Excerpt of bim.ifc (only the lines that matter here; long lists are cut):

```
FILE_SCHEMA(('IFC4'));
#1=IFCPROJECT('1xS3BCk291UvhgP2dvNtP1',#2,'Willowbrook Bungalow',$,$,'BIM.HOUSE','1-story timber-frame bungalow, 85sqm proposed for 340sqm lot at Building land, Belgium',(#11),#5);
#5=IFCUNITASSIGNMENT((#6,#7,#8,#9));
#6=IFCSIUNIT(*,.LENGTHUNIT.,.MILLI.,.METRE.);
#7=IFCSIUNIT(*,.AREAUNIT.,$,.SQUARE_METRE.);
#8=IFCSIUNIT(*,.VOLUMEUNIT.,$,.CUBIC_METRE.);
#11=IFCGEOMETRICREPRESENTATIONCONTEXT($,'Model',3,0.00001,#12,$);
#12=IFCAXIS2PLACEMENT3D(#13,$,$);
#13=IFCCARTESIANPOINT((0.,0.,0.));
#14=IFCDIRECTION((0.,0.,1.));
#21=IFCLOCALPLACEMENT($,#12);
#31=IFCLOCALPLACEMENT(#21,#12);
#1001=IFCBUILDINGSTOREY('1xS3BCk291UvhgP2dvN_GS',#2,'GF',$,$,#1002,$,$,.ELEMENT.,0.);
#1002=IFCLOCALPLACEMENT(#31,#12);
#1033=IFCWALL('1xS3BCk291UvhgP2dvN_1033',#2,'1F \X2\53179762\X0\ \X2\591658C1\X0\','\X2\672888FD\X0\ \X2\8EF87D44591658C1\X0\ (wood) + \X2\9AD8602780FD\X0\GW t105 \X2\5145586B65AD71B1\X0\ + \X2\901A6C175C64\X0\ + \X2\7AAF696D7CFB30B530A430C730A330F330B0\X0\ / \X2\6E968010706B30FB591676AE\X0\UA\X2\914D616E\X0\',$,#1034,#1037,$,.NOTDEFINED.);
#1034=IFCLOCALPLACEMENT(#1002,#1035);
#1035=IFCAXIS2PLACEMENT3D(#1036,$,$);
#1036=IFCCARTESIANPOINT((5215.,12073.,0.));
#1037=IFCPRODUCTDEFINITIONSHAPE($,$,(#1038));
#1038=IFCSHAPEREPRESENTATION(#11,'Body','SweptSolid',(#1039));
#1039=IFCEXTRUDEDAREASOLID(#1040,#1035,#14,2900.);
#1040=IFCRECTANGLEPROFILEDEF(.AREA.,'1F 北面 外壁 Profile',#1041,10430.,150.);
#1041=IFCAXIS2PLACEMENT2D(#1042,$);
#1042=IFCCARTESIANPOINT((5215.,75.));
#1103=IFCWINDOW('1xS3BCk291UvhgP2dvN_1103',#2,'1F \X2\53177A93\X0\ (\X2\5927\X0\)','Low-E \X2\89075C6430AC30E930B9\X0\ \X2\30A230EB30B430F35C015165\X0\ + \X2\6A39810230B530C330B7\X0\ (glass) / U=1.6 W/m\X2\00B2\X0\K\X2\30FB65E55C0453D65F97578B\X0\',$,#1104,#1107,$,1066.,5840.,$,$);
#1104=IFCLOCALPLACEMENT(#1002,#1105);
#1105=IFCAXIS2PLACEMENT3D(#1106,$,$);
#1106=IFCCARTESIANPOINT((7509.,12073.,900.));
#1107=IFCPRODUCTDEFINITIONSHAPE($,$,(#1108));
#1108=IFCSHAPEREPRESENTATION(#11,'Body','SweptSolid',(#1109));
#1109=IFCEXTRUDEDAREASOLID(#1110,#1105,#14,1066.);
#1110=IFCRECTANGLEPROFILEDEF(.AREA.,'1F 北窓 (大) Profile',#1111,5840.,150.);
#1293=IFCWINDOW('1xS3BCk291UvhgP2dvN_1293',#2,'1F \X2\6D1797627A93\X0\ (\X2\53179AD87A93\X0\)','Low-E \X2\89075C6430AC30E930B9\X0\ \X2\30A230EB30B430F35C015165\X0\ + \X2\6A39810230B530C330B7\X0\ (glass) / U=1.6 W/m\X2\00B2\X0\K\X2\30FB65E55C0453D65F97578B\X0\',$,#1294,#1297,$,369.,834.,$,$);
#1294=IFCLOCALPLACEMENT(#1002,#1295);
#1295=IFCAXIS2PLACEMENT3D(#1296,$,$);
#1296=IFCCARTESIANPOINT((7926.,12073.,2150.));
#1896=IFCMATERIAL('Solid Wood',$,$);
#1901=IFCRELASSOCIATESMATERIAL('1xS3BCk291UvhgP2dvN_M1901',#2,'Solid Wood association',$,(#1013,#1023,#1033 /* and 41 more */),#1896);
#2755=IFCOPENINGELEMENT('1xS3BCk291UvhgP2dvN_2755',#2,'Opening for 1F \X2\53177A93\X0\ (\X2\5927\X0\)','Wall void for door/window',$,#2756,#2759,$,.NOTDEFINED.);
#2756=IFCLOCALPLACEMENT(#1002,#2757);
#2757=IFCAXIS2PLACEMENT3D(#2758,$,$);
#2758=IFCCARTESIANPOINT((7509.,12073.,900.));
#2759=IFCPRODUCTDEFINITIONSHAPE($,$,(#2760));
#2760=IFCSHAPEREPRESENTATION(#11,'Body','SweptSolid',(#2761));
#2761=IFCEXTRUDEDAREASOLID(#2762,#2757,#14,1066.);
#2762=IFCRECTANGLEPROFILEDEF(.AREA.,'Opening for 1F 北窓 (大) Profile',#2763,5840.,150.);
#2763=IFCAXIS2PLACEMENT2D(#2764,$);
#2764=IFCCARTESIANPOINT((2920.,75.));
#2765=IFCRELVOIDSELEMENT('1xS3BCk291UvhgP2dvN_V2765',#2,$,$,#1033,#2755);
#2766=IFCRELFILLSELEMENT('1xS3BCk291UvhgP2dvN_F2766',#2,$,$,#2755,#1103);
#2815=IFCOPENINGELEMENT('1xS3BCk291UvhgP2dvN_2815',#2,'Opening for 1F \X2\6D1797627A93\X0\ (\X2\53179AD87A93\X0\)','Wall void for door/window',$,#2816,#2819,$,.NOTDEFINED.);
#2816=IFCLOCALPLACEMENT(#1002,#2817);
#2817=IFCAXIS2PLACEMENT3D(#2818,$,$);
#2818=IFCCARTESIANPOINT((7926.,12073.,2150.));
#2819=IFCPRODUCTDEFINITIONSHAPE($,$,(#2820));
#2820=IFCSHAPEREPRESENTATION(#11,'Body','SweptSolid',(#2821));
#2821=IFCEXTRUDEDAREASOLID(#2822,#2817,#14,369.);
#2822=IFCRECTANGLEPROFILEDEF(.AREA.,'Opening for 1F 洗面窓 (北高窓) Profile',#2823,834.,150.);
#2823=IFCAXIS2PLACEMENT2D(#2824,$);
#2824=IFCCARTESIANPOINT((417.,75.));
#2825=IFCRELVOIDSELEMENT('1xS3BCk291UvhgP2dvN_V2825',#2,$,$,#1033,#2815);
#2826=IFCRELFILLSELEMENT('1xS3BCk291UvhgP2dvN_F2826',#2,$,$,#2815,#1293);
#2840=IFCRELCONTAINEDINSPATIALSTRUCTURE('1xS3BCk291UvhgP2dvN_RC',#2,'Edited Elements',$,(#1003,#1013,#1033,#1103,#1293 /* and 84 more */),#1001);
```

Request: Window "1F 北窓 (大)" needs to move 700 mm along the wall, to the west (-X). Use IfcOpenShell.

```python
import ifcopenshell
import ifcopenshell.api.geometry
import ifcopenshell.util.placement
import ifcopenshell.util.unit

model = ifcopenshell.open("bim.ifc")
unit_scale = ifcopenshell.util.unit.calculate_unit_scale(model)

window = model.by_id(1103)
opening = window.FillsVoids[0].RelatingOpeningElement
wall = opening.VoidsElements[0].RelatingBuildingElement

wall_matrix = ifcopenshell.util.placement.get_local_placement(wall.ObjectPlacement)
shift = wall_matrix[:3, 0] * -0.7 / unit_scale
before = ifcopenshell.util.placement.get_local_placement(window.ObjectPlacement)[:3, 3].copy()

# The window is not placed relative to its opening, so move both.
for product in (opening, window):
    matrix = ifcopenshell.util.placement.get_local_placement(product.ObjectPlacement)
    matrix[:3, 3] += shift
    ifcopenshell.api.geometry.edit_object_placement(model, product=product, matrix=matrix, is_si=False)

after = ifcopenshell.util.placement.get_local_placement(window.ObjectPlacement)[:3, 3]
print("window moved by", (after - before).round(3) + 0.0)

model.write("bim_v2.ifc")
```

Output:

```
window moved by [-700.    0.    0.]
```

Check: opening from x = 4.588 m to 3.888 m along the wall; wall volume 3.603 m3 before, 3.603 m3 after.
